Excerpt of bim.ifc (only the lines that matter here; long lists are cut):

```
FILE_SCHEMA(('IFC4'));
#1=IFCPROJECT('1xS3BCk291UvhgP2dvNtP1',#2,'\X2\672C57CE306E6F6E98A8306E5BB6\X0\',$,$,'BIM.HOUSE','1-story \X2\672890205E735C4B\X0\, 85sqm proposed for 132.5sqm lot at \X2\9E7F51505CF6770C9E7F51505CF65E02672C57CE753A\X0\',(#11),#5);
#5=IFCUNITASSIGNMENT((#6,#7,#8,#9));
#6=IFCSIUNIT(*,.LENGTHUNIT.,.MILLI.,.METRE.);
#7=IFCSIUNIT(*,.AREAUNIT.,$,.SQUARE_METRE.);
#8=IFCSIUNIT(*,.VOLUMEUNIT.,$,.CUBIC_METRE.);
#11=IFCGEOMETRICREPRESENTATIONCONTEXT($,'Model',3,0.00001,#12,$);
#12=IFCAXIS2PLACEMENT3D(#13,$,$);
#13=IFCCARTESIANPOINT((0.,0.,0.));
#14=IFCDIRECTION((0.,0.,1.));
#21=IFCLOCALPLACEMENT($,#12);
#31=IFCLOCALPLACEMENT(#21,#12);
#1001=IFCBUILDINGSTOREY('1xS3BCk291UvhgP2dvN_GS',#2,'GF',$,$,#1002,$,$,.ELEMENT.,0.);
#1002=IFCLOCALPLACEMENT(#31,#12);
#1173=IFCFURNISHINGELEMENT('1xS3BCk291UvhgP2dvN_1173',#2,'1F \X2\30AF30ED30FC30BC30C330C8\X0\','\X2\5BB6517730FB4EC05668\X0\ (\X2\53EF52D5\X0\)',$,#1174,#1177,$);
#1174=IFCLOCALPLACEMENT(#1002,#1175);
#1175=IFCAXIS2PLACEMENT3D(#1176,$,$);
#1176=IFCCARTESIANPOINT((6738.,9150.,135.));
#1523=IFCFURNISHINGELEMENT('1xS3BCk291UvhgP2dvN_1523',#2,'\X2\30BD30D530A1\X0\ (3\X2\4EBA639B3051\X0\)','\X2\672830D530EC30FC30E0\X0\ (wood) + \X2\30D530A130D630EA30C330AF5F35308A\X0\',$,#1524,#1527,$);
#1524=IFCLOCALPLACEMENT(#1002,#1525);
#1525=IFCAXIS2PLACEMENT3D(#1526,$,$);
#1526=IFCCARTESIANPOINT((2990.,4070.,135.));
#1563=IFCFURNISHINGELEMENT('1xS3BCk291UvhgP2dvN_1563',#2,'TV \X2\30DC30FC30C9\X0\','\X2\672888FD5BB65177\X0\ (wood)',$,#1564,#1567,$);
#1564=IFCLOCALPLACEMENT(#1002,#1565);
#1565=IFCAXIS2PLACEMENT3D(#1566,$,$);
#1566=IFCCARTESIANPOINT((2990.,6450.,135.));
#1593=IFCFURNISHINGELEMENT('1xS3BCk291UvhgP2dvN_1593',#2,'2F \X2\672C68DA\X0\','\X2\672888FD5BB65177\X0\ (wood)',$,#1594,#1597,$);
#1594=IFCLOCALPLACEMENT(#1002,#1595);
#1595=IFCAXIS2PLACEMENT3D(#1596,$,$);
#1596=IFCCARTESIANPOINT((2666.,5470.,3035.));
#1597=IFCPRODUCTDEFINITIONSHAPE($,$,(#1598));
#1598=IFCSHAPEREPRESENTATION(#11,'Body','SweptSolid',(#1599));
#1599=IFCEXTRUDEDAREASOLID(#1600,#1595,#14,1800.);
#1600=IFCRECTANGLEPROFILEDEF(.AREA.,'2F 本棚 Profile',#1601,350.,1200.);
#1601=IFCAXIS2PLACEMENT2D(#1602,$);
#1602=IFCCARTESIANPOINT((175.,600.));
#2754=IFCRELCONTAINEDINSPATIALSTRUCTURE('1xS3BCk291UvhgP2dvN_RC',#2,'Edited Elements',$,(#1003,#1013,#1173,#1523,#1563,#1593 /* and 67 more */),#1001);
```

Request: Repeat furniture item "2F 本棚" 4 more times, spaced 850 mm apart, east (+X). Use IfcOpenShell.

```python
import numpy as np
import ifcopenshell
import ifcopenshell.api.geometry
import ifcopenshell.api.root
import ifcopenshell.util.element
import ifcopenshell.util.placement
import ifcopenshell.util.unit

model = ifcopenshell.open("bim.ifc")
unit_scale = ifcopenshell.util.unit.calculate_unit_scale(model)


def reuse_history(source, copy):
    """copy_class also copies each property set's owner history, people and application; keep the originals."""
    for rel in copy.IsDefinedBy:
        if rel.is_a("IfcRelDefinesByProperties") and (history := rel.RelatingPropertyDefinition.OwnerHistory):
            rel.RelatingPropertyDefinition.OwnerHistory = source.OwnerHistory
            ifcopenshell.util.element.remove_deep2(model, history)


source = model.by_guid("1xS3BCk291UvhgP2dvN_1593")
base = ifcopenshell.util.placement.get_local_placement(source.ObjectPlacement)
step = np.array([1.0, 0.0, 0.0]) * 0.85 / unit_scale

for i in range(1, 5):
    copy = ifcopenshell.api.root.copy_class(model, product=source)
    copy.Representation = ifcopenshell.util.element.copy_deep(
        model, source.Representation, exclude=["IfcGeometricRepresentationContext", "IfcRepresentationMap"]
    )
    reuse_history(source, copy)
    matrix = base.copy()
    matrix[:3, 3] += i * step
    print("added at", matrix[:3, 3].round(3) + 0.0)
    ifcopenshell.api.geometry.edit_object_placement(model, product=copy, matrix=matrix, is_si=False)

model.write("bim_v2.ifc")
```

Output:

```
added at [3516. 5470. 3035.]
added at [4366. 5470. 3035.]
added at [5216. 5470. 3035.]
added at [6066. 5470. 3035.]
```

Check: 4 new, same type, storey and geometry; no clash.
